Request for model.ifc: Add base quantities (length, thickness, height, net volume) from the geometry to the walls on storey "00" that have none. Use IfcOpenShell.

First a look at what the model holds.

```python
import ifcopenshell
import ifcopenshell.util.element
import ifcopenshell.util.unit

model = ifcopenshell.open("model.ifc")
print(model.schema)
for unit_type in ("LENGTHUNIT", "AREAUNIT", "VOLUMEUNIT"):
    print(unit_type, ifcopenshell.util.unit.calculate_unit_scale(model, unit_type))
storey = next(s for s in model.by_type("IfcBuildingStorey") if s.Name == "00")
walls = [e for e in ifcopenshell.util.element.get_decomposition(storey) if e.is_a("IfcWall")]
for e in sorted(walls, key=lambda e: e.id()):
    print(e.id(), e.is_a(), e.Name, list(ifcopenshell.util.element.get_psets(e, qtos_only=True)), sep=" | ")
```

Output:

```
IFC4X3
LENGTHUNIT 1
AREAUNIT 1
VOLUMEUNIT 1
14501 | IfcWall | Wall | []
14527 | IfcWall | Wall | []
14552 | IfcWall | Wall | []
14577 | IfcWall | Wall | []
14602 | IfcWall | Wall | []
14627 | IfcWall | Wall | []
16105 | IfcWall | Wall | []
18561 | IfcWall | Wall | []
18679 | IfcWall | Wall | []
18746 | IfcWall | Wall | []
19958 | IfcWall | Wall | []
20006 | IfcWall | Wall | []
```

```python
import ifcopenshell
import ifcopenshell.api.pset
import ifcopenshell.geom
import ifcopenshell.util.element
import ifcopenshell.util.shape
import ifcopenshell.util.unit

model = ifcopenshell.open("model.ifc")
unit_scale = ifcopenshell.util.unit.calculate_unit_scale(model)
volume_scale = ifcopenshell.util.unit.calculate_unit_scale(model, "VOLUMEUNIT")
settings = ifcopenshell.geom.settings()

storey = next(s for s in model.by_type("IfcBuildingStorey") if s.Name == "00")
walls = [e for e in ifcopenshell.util.element.get_decomposition(storey) if e.is_a("IfcWall")]

for e in sorted(walls, key=lambda e: e.id()):
    if ifcopenshell.util.element.get_psets(e, qtos_only=True, should_inherit=False):
        continue
    # Geometry comes back in metres, in the element's own axes.
    shape = ifcopenshell.geom.create_shape(settings, e)
    values = {
        "Length": ifcopenshell.util.shape.get_x(shape.geometry) / unit_scale,
        "Width": ifcopenshell.util.shape.get_y(shape.geometry) / unit_scale,
        "Height": ifcopenshell.util.shape.get_z(shape.geometry) / unit_scale,
        "NetVolume": ifcopenshell.util.shape.get_volume(shape.geometry) / volume_scale,
    }
    qto = ifcopenshell.api.pset.add_qto(model, product=e, name="Qto_WallBaseQuantities")
    ifcopenshell.api.pset.edit_qto(model, qto=qto, properties=values)
    print(e.id(), {k: round(v, 3) for k, v in values.items()})

model.write("model_rev.ifc")
```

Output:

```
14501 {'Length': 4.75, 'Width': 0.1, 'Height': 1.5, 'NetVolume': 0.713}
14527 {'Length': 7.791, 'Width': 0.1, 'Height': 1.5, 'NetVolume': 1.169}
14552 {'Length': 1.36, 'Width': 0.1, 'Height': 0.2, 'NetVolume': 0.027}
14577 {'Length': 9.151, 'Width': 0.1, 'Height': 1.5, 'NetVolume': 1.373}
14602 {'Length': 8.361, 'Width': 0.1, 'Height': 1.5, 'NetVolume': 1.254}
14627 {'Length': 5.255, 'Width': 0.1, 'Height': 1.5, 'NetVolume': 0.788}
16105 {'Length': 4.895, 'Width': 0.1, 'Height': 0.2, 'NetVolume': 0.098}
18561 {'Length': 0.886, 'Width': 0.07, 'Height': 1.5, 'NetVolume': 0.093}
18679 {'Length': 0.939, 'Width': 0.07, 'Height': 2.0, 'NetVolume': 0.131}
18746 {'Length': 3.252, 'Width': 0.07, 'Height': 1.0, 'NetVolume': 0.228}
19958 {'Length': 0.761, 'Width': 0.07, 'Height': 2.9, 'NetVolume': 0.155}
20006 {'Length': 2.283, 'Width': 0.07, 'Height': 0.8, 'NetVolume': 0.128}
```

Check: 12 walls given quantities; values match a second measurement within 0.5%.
